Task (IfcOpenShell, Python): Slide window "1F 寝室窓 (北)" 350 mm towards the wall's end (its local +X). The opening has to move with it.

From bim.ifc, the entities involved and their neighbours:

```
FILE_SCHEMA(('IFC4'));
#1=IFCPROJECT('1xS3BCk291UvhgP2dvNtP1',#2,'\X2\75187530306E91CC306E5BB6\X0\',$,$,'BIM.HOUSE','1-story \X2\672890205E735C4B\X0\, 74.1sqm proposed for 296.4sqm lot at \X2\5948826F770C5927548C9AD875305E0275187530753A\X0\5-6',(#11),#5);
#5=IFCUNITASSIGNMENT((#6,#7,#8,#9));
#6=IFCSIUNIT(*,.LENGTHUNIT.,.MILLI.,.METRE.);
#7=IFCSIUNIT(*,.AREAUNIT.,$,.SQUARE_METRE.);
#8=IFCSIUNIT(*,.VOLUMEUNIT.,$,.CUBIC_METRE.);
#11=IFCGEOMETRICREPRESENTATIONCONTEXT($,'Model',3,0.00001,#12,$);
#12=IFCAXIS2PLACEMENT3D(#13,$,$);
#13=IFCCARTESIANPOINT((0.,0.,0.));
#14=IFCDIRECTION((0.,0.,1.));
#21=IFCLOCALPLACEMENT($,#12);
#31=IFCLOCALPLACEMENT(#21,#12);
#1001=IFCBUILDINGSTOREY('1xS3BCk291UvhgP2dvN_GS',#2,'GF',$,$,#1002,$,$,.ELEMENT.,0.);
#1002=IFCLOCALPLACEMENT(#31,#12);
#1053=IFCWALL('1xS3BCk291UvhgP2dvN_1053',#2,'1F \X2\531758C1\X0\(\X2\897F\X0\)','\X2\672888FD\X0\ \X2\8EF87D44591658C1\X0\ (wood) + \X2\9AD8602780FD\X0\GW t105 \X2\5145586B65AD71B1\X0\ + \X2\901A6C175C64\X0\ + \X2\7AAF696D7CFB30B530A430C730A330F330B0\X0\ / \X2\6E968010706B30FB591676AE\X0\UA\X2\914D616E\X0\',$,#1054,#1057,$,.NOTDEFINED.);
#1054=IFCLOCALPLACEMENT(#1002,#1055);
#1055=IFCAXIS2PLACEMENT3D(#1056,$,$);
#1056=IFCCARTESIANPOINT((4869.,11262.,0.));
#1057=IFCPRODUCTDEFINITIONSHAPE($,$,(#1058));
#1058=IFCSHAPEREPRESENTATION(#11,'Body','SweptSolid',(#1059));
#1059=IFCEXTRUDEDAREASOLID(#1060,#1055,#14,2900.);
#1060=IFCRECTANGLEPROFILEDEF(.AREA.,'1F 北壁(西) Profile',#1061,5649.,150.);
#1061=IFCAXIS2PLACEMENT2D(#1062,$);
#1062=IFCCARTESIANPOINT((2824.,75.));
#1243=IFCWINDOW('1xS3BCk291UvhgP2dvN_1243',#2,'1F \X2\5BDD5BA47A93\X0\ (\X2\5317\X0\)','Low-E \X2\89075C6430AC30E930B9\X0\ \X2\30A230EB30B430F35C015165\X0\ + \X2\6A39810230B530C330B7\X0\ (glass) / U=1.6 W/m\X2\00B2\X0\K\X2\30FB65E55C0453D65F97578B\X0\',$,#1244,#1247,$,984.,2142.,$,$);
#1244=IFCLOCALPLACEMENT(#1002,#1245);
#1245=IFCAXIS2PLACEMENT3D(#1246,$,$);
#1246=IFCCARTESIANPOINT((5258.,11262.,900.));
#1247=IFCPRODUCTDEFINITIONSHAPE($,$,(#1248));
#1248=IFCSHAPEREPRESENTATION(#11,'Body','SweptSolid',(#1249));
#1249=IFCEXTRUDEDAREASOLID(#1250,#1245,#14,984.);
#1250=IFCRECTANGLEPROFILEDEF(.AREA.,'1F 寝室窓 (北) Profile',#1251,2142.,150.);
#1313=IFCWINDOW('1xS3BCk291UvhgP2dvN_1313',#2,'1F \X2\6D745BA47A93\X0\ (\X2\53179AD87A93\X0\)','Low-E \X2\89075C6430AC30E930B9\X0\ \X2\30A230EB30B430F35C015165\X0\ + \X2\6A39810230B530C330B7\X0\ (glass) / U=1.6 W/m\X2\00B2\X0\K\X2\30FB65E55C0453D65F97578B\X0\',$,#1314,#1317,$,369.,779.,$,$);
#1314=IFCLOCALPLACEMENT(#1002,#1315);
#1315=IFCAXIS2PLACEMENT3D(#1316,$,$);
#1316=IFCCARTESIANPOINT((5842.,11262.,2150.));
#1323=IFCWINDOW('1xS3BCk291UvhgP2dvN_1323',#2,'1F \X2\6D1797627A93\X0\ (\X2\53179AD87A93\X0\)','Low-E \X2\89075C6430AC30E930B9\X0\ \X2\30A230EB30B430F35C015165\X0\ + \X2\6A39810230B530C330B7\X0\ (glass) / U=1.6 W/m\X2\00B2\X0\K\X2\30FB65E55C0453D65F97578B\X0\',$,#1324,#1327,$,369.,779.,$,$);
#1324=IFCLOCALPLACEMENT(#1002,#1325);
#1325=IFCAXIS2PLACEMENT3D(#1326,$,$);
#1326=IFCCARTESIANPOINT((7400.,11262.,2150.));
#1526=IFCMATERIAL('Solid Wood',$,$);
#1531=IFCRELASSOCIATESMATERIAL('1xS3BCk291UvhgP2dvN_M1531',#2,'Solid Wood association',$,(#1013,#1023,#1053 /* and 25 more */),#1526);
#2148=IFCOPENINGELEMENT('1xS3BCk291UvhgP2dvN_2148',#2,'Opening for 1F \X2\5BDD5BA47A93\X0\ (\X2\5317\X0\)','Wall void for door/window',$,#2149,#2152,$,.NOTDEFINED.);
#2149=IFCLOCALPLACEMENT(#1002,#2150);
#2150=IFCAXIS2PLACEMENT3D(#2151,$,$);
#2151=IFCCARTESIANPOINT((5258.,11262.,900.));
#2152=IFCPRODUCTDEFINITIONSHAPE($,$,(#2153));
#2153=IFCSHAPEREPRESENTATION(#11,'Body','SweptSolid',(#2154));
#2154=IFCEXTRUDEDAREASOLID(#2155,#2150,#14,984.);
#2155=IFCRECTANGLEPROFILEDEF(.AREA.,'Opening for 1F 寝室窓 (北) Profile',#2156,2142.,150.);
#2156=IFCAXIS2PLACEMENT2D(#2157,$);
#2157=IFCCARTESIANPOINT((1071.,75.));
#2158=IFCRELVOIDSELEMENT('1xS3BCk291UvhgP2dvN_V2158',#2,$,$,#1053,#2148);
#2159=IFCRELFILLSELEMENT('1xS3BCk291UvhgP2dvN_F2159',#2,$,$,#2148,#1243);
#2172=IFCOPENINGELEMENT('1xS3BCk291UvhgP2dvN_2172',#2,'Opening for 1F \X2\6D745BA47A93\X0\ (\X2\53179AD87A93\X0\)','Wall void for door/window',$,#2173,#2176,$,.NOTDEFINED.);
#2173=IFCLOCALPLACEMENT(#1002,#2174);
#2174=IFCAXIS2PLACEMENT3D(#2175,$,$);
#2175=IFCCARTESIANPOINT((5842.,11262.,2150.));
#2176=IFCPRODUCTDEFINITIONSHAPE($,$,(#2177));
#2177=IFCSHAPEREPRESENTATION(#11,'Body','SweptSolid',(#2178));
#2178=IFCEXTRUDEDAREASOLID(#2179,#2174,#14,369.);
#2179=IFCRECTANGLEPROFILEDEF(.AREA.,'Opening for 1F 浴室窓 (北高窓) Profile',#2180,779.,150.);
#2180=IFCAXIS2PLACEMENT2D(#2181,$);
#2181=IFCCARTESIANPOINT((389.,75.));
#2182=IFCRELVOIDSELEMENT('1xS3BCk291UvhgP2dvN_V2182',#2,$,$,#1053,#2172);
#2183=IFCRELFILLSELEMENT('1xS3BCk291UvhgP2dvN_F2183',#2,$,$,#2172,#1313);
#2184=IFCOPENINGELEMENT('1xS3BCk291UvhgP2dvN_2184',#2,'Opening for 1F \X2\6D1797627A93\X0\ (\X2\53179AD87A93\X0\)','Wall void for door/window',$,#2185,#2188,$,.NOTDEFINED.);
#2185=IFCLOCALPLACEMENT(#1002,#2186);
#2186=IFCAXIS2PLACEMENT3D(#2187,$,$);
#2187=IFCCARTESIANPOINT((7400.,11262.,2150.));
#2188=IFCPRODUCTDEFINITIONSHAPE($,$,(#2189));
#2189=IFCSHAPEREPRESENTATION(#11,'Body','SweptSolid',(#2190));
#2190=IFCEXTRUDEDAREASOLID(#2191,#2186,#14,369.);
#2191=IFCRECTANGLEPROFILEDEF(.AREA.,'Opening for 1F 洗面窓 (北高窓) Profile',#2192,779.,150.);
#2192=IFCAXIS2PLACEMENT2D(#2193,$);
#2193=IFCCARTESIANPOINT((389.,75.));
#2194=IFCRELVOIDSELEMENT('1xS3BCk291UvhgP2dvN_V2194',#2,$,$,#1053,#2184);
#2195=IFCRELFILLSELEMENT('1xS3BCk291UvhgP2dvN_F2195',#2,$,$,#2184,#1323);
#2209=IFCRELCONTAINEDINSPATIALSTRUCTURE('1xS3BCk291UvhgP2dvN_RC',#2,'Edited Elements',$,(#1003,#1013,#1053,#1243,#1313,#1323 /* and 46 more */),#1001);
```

```python
import ifcopenshell
import ifcopenshell.api.geometry
import ifcopenshell.util.placement

model = ifcopenshell.open("bim.ifc")

window = model.by_guid("1xS3BCk291UvhgP2dvN_1243")
opening = window.FillsVoids[0].RelatingOpeningElement
wall = opening.VoidsElements[0].RelatingBuildingElement

wall_matrix = ifcopenshell.util.placement.get_local_placement(wall.ObjectPlacement)
shift = wall_matrix[:3, 0] * 350.0
before = ifcopenshell.util.placement.get_local_placement(window.ObjectPlacement)[:3, 3].copy()

# The window is not placed relative to its opening, so move both.
for product in (opening, window):
    matrix = ifcopenshell.util.placement.get_local_placement(product.ObjectPlacement)
    matrix[:3, 3] += shift
    ifcopenshell.api.geometry.edit_object_placement(model, product=product, matrix=matrix, is_si=False)

after = ifcopenshell.util.placement.get_local_placement(window.ObjectPlacement)[:3, 3]
print("window moved by", (after - before).round(3) + 0.0)

model.write("bim-out.ifc")
```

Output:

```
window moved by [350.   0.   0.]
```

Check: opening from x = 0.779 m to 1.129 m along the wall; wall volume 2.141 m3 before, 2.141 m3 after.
